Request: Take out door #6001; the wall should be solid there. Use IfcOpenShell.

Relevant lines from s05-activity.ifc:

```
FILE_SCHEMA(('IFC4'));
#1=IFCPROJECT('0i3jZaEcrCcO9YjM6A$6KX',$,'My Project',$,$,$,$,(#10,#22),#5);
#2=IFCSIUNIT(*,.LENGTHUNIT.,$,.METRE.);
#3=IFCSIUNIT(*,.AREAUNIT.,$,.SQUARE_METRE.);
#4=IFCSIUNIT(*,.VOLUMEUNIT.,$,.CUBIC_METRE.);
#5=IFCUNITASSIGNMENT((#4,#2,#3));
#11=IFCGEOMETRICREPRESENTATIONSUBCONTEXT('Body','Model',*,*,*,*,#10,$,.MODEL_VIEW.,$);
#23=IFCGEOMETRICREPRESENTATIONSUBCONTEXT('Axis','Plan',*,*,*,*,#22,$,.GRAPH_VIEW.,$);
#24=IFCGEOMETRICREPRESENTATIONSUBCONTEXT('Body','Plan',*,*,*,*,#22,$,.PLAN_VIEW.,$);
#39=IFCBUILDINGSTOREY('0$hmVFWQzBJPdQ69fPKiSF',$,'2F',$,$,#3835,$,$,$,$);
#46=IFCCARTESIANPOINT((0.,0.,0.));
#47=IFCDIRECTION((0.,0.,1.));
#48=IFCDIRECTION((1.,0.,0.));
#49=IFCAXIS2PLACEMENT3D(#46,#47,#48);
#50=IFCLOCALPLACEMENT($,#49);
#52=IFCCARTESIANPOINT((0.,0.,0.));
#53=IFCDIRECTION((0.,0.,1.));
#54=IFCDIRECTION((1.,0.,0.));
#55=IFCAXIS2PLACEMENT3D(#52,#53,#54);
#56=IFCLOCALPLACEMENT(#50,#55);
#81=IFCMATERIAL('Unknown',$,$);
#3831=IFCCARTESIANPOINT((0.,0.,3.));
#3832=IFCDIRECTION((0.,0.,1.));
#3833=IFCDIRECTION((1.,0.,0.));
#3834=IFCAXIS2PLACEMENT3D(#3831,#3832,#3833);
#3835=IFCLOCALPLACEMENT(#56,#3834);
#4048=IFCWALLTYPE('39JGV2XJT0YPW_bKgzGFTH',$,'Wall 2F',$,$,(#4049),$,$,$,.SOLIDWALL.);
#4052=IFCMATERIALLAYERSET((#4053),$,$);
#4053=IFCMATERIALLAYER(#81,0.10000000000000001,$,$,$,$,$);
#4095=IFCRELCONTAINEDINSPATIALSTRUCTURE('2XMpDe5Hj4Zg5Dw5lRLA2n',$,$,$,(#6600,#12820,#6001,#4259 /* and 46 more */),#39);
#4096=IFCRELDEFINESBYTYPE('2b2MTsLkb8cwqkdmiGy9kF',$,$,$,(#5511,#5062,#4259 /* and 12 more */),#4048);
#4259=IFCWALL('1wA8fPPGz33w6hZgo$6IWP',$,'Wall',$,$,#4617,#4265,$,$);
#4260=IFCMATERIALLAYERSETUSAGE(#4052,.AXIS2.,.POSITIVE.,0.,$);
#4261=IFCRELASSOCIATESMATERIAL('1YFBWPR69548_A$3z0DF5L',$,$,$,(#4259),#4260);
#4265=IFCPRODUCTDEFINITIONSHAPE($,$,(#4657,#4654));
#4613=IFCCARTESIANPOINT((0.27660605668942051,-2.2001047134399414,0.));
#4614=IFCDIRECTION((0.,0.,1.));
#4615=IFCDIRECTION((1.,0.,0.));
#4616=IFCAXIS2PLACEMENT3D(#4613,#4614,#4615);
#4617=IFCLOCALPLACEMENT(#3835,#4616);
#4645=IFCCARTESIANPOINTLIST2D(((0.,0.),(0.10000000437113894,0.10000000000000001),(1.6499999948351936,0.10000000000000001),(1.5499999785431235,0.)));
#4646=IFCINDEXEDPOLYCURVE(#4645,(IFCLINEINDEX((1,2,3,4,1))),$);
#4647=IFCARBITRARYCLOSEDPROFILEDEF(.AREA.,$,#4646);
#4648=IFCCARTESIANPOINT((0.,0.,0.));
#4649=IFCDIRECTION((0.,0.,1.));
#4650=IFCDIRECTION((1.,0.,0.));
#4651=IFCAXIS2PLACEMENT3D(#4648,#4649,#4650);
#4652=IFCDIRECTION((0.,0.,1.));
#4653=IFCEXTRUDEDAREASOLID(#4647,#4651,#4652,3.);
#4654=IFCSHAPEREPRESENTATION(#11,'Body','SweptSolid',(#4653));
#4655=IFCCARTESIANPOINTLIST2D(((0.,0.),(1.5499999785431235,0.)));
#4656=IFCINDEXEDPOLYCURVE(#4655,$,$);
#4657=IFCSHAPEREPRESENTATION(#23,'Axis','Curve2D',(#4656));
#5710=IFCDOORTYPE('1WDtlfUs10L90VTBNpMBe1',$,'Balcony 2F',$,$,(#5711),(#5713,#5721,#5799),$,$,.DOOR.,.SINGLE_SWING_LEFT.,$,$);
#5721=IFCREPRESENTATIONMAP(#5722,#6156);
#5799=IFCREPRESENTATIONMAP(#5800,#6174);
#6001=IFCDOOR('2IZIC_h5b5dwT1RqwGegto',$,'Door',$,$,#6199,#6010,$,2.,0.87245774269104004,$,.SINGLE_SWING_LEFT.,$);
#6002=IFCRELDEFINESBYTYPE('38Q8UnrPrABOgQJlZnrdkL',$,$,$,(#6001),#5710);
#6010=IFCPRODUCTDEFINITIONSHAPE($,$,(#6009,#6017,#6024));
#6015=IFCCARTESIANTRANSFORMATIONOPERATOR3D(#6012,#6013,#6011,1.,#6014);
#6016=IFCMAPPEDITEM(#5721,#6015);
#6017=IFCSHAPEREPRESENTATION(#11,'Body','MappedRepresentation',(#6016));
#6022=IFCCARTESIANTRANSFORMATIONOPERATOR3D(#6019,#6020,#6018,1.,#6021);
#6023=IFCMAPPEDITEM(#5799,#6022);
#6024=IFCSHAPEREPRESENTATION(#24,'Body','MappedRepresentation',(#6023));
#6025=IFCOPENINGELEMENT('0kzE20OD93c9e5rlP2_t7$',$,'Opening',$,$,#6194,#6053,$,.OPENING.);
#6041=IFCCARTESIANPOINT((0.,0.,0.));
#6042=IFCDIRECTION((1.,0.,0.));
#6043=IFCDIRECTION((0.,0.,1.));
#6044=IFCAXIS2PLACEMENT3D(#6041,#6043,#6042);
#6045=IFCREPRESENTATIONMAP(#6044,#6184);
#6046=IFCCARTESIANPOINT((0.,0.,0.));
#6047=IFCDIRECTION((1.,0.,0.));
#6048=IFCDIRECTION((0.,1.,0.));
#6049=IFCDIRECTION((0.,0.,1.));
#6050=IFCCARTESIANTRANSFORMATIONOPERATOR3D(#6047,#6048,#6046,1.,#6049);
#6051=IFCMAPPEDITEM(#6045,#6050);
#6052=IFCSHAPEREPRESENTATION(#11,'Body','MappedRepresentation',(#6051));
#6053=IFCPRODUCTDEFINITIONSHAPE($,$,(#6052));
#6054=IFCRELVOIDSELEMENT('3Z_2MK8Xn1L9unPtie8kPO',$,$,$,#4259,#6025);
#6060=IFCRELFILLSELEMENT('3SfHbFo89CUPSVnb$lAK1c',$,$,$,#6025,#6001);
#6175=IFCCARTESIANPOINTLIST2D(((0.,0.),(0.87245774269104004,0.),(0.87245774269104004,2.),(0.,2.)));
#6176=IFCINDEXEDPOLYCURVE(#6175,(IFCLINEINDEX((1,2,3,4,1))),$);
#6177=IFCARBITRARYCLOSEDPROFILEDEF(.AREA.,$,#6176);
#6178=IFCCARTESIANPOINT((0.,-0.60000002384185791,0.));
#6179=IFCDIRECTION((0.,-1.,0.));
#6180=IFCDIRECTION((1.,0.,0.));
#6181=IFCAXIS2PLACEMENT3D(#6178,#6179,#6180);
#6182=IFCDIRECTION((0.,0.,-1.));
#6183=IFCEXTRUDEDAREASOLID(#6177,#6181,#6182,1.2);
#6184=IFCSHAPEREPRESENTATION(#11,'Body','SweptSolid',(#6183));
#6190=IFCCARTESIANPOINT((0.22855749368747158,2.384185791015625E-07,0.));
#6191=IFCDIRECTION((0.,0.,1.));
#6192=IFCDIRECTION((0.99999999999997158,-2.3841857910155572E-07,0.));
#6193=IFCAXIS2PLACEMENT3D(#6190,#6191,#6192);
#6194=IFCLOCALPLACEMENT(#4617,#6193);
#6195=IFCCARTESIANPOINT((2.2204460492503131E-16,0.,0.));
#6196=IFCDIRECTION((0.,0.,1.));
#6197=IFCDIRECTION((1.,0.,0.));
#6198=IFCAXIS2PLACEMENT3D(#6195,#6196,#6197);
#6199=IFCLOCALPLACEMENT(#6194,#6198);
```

```python
import ifcopenshell
import ifcopenshell.api.feature
import ifcopenshell.api.root
import ifcopenshell.geom
import ifcopenshell.util.shape

model = ifcopenshell.open("s05-activity.ifc")
settings = ifcopenshell.geom.settings()


def volume(element):
    """Net volume in cubic metres, openings subtracted."""
    shape = ifcopenshell.geom.create_shape(settings, element)
    return ifcopenshell.util.shape.get_volume(shape.geometry)


door = model.by_guid("2IZIC_h5b5dwT1RqwGegto")
opening = door.FillsVoids[0].RelatingOpeningElement
wall = opening.VoidsElements[0].RelatingBuildingElement
before = volume(wall)

ifcopenshell.api.root.remove_product(model, product=door)
ifcopenshell.api.feature.remove_feature(model, feature=opening)

after = volume(wall)

print(f"wall volume {before:.3f} -> {after:.3f} m3")

model.write("s05-activity_rev.ifc")
```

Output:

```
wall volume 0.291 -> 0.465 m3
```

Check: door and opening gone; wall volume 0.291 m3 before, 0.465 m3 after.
